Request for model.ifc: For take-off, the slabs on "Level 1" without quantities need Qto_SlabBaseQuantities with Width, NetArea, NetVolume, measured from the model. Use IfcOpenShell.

First a look at what the model holds.

```python
import ifcopenshell
import ifcopenshell.util.element
import ifcopenshell.util.unit

model = ifcopenshell.open("model.ifc")
print(model.schema)
for unit_type in ("LENGTHUNIT", "AREAUNIT", "VOLUMEUNIT"):
    print(unit_type, ifcopenshell.util.unit.calculate_unit_scale(model, unit_type))
storey = next(s for s in model.by_type("IfcBuildingStorey") if s.Name == "Level 1")
slabs = [e for e in ifcopenshell.util.element.get_decomposition(storey) if e.is_a("IfcSlab")]
for e in sorted(slabs, key=lambda e: e.id()):
    print(e.id(), e.is_a(), e.Name, list(ifcopenshell.util.element.get_psets(e, qtos_only=True)), sep=" | ")
```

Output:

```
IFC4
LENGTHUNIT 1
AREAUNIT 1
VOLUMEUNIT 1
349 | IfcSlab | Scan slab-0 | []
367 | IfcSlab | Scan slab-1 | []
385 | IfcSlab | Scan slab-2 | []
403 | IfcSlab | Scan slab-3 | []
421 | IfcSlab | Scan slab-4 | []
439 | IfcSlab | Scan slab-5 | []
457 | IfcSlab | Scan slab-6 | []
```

```python
import ifcopenshell
import ifcopenshell.api.pset
import ifcopenshell.geom
import ifcopenshell.util.element
import ifcopenshell.util.shape
import ifcopenshell.util.unit

model = ifcopenshell.open("model.ifc")
unit_scale = ifcopenshell.util.unit.calculate_unit_scale(model)
area_scale = ifcopenshell.util.unit.calculate_unit_scale(model, "AREAUNIT")
volume_scale = ifcopenshell.util.unit.calculate_unit_scale(model, "VOLUMEUNIT")
settings = ifcopenshell.geom.settings()

storey = next(s for s in model.by_type("IfcBuildingStorey") if s.Name == "Level 1")
slabs = [e for e in ifcopenshell.util.element.get_decomposition(storey) if e.is_a("IfcSlab")]

for e in sorted(slabs, key=lambda e: e.id()):
    if ifcopenshell.util.element.get_psets(e, qtos_only=True, should_inherit=False):
        continue
    # Geometry comes back in metres, in the element's own axes.
    shape = ifcopenshell.geom.create_shape(settings, e)
    values = {
        "Width": ifcopenshell.util.shape.get_z(shape.geometry) / unit_scale,
        "NetArea": ifcopenshell.util.shape.get_footprint_area(shape.geometry) / area_scale,
        "NetVolume": ifcopenshell.util.shape.get_volume(shape.geometry) / volume_scale,
    }
    qto = ifcopenshell.api.pset.add_qto(model, product=e, name="Qto_SlabBaseQuantities")
    ifcopenshell.api.pset.edit_qto(model, qto=qto, properties=values)
    print(e.id(), {k: round(v, 3) for k, v in values.items()})

model.write("model_edited.ifc")
```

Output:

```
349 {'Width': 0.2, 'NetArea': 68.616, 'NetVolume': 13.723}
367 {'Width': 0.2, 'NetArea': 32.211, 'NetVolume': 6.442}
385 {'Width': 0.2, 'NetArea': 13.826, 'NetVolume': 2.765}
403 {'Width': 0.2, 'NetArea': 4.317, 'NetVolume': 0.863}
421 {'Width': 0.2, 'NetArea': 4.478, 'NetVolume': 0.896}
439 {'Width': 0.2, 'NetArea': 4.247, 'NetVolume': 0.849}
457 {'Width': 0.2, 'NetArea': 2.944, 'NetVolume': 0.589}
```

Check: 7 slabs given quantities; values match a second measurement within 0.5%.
